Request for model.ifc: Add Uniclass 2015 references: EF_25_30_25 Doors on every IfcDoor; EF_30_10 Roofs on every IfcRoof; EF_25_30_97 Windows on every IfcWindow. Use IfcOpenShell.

First a look at what the model holds.

```python
import ifcopenshell

model = ifcopenshell.open("model.ifc")
print(model.schema)
print("classifications:", [c.Name for c in model.by_type("IfcClassification")])
for ifc_class in ("IfcDoor", "IfcRoof", "IfcStair", "IfcWall", "IfcWindow"):
    print(ifc_class, len(model.by_type(ifc_class)))
```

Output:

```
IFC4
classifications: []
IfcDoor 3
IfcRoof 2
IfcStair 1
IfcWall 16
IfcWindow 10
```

```python
import ifcopenshell
import ifcopenshell.api.classification

model = ifcopenshell.open("model.ifc")

system = ifcopenshell.api.classification.add_classification(model, classification="Uniclass 2015")

codes = {
    "IfcDoor": ("EF_25_30_25", "Doors"),
    "IfcRoof": ("EF_30_10", "Roofs"),
    "IfcWindow": ("EF_25_30_97", "Windows"),
}
for ifc_class, (code, name) in codes.items():
    products = model.by_type(ifc_class)
    ifcopenshell.api.classification.add_reference(
        model, products=products, classification=system, identification=code, name=name
    )
    print(code, len(products))

model.write("model-out.ifc")
```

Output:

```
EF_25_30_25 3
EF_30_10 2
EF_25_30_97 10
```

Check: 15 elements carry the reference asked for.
